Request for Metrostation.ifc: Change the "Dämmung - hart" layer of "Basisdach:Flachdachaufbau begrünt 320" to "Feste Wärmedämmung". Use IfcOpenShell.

First a look at what the model holds.

```python
import ifcopenshell
import ifcopenshell.util.element

model = ifcopenshell.open("Metrostation.ifc")
print(model.schema)
for layer_set in model.by_type("IfcMaterialLayerSet"):
    if layer_set.LayerSetName == "Basisdach:Flachdachaufbau begrünt 320":
        for layer in layer_set.MaterialLayers:
            print(layer.id(), layer.Material and layer.Material.Name, layer.LayerThickness, sep=" | ")
        print(len(ifcopenshell.util.element.get_elements_by_material(model, layer_set)), "elements and types use it")
print(sorted(m.Name for m in model.by_type("IfcMaterial") if m.Name)[:60])
```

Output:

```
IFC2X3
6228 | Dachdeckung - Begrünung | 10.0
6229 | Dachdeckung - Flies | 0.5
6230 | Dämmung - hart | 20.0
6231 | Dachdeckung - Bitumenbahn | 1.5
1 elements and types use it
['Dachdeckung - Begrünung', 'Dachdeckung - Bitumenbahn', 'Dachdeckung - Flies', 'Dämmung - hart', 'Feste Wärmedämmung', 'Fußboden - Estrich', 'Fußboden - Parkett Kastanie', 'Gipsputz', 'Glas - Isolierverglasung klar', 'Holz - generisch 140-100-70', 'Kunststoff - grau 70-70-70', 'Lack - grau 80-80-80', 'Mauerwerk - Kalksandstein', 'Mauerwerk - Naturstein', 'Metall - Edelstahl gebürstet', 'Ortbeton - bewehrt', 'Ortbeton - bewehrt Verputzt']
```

```python
import ifcopenshell
import ifcopenshell.api.material

model = ifcopenshell.open("Metrostation.ifc")

layer_set = next(s for s in model.by_type("IfcMaterialLayerSet") if s.LayerSetName == "Basisdach:Flachdachaufbau begrünt 320")
layer = next(l for l in layer_set.MaterialLayers if l.Material and l.Material.Name == "Dämmung - hart")
material = next(m for m in model.by_type("IfcMaterial") if m.Name == "Feste Wärmedämmung")

# Point this one layer at the other material; renaming the old one would change it everywhere.
ifcopenshell.api.material.edit_layer(model, layer=layer, attributes={}, material=material)

print([l.Material.Name if l.Material else None for l in layer_set.MaterialLayers])

model.write("Metrostation-out.ifc")
```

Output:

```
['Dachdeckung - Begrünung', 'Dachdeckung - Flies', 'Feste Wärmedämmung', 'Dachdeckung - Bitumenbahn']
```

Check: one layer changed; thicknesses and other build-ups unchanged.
